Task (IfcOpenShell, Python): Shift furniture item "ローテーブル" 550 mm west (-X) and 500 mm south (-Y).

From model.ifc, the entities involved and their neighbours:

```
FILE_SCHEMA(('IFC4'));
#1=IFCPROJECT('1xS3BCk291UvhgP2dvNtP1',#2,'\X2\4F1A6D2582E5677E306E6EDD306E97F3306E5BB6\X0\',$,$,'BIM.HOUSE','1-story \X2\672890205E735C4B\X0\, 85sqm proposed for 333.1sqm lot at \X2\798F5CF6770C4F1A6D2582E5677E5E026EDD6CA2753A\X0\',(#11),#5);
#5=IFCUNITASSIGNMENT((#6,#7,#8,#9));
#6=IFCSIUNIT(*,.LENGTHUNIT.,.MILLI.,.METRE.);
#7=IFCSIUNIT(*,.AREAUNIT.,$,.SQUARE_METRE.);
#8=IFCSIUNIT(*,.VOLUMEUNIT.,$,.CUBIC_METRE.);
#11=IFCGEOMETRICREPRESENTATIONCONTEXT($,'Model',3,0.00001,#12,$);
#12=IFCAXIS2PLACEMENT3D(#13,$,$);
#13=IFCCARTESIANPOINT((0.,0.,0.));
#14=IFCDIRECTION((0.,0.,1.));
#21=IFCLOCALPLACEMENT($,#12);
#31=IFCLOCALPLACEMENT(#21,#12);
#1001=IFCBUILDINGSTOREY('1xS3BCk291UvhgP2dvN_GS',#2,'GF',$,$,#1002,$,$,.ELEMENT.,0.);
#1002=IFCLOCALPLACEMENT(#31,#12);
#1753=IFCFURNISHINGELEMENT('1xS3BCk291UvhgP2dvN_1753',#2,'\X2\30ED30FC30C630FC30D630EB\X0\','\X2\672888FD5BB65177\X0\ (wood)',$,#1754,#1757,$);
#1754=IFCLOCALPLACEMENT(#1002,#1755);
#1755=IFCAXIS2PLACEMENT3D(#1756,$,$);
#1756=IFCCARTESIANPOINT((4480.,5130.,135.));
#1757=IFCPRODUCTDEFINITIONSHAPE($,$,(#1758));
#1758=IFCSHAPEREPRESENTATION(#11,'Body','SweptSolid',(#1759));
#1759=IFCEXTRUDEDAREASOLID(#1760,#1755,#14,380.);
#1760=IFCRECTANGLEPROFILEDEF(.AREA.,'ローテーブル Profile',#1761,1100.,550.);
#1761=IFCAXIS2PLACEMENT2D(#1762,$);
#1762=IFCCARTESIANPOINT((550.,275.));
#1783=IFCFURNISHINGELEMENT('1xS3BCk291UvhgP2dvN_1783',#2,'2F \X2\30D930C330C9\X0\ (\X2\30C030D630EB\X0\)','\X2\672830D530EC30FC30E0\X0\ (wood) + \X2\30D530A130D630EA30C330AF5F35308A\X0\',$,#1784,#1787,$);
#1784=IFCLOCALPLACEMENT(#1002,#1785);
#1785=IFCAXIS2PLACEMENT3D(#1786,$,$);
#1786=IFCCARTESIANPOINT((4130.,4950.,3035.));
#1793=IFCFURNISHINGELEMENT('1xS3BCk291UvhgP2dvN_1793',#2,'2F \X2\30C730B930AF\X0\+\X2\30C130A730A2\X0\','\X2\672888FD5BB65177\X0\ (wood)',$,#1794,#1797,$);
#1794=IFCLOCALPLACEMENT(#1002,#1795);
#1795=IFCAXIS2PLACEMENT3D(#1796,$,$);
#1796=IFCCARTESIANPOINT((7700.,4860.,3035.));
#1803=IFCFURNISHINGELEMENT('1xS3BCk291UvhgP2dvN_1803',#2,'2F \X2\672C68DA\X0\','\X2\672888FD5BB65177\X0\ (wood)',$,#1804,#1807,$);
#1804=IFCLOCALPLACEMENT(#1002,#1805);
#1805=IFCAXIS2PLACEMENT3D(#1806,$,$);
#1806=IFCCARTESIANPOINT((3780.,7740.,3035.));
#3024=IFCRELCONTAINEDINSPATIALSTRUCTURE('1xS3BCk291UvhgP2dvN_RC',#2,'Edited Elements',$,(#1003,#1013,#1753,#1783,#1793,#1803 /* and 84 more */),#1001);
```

```python
import ifcopenshell
import ifcopenshell.api.geometry
import ifcopenshell.util.placement

model = ifcopenshell.open("model.ifc")

item = model.by_guid("1xS3BCk291UvhgP2dvN_1753")
matrix = ifcopenshell.util.placement.get_local_placement(item.ObjectPlacement)
matrix[0, 3] -= 550.0
matrix[1, 3] -= 500.0
ifcopenshell.api.geometry.edit_object_placement(model, product=item, matrix=matrix, is_si=False)

print(ifcopenshell.util.placement.get_local_placement(item.ObjectPlacement).round(3) + 0.0)

model.write("model_rev.ifc")
```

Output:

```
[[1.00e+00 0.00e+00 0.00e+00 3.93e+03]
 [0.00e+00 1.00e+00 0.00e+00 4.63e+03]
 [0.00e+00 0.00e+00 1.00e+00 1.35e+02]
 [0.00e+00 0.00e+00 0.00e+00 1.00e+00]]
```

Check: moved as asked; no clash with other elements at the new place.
